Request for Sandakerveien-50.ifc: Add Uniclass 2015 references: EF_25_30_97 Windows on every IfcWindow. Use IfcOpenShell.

First a look at what the model holds.

```python
import ifcopenshell

model = ifcopenshell.open("Sandakerveien-50.ifc")
print(model.schema)
print("classifications:", [c.Name for c in model.by_type("IfcClassification")])
for ifc_class in ("IfcDoor", "IfcRoof", "IfcStair", "IfcWall", "IfcWindow"):
    print(ifc_class, len(model.by_type(ifc_class)))
```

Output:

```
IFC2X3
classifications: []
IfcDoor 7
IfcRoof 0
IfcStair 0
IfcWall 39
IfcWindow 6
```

```python
import ifcopenshell
import ifcopenshell.api.classification

model = ifcopenshell.open("Sandakerveien-50.ifc")

# IFC2X3 requires Source and Edition and has no link from the project to the system.
system = model.create_entity("IfcClassification", Source="NBS", Edition="2015", Name="Uniclass 2015")

codes = {
    "IfcWindow": ("EF_25_30_97", "Windows"),
}
for ifc_class, (code, name) in codes.items():
    products = model.by_type(ifc_class)
    ifcopenshell.api.classification.add_reference(
        model, products=products, classification=system, identification=code, name=name
    )
    print(code, len(products))

model.write("Sandakerveien-50_rev.ifc")
```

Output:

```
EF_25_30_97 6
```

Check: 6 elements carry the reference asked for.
